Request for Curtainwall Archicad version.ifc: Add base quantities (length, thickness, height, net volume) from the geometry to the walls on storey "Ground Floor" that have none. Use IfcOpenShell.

First a look at what the model holds.

```python
import ifcopenshell
import ifcopenshell.util.element
import ifcopenshell.util.unit

model = ifcopenshell.open("Curtainwall Archicad version.ifc")
print(model.schema)
for unit_type in ("LENGTHUNIT", "AREAUNIT", "VOLUMEUNIT"):
    print(unit_type, ifcopenshell.util.unit.calculate_unit_scale(model, unit_type))
storey = next(s for s in model.by_type("IfcBuildingStorey") if s.Name == "Ground Floor")
walls = [e for e in ifcopenshell.util.element.get_decomposition(storey) if e.is_a("IfcWall")]
for e in sorted(walls, key=lambda e: e.id()):
    print(e.id(), e.is_a(), e.Name, list(ifcopenshell.util.element.get_psets(e, qtos_only=True)), sep=" | ")
```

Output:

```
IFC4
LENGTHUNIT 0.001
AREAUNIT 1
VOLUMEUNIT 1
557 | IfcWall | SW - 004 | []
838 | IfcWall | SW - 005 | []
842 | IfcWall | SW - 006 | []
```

```python
import ifcopenshell
import ifcopenshell.api.pset
import ifcopenshell.geom
import ifcopenshell.util.element
import ifcopenshell.util.shape
import ifcopenshell.util.unit

model = ifcopenshell.open("Curtainwall Archicad version.ifc")
unit_scale = ifcopenshell.util.unit.calculate_unit_scale(model)
volume_scale = ifcopenshell.util.unit.calculate_unit_scale(model, "VOLUMEUNIT")
settings = ifcopenshell.geom.settings()

storey = next(s for s in model.by_type("IfcBuildingStorey") if s.Name == "Ground Floor")
walls = [e for e in ifcopenshell.util.element.get_decomposition(storey) if e.is_a("IfcWall")]

for e in sorted(walls, key=lambda e: e.id()):
    if ifcopenshell.util.element.get_psets(e, qtos_only=True, should_inherit=False):
        continue
    # Geometry comes back in metres, in the element's own axes.
    shape = ifcopenshell.geom.create_shape(settings, e)
    values = {
        "Length": ifcopenshell.util.shape.get_x(shape.geometry) / unit_scale,
        "Width": ifcopenshell.util.shape.get_y(shape.geometry) / unit_scale,
        "Height": ifcopenshell.util.shape.get_z(shape.geometry) / unit_scale,
        "NetVolume": ifcopenshell.util.shape.get_volume(shape.geometry) / volume_scale,
    }
    qto = ifcopenshell.api.pset.add_qto(model, product=e, name="Qto_WallBaseQuantities")
    ifcopenshell.api.pset.edit_qto(model, qto=qto, properties=values)
    print(e.id(), {k: round(v, 3) for k, v in values.items()})

model.write("Curtainwall Archicad version_edited.ifc")
```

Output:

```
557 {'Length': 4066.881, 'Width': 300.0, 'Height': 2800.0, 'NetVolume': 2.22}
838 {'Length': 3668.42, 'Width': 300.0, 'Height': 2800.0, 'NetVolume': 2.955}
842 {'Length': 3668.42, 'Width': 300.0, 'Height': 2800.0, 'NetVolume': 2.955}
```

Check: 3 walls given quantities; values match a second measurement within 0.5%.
